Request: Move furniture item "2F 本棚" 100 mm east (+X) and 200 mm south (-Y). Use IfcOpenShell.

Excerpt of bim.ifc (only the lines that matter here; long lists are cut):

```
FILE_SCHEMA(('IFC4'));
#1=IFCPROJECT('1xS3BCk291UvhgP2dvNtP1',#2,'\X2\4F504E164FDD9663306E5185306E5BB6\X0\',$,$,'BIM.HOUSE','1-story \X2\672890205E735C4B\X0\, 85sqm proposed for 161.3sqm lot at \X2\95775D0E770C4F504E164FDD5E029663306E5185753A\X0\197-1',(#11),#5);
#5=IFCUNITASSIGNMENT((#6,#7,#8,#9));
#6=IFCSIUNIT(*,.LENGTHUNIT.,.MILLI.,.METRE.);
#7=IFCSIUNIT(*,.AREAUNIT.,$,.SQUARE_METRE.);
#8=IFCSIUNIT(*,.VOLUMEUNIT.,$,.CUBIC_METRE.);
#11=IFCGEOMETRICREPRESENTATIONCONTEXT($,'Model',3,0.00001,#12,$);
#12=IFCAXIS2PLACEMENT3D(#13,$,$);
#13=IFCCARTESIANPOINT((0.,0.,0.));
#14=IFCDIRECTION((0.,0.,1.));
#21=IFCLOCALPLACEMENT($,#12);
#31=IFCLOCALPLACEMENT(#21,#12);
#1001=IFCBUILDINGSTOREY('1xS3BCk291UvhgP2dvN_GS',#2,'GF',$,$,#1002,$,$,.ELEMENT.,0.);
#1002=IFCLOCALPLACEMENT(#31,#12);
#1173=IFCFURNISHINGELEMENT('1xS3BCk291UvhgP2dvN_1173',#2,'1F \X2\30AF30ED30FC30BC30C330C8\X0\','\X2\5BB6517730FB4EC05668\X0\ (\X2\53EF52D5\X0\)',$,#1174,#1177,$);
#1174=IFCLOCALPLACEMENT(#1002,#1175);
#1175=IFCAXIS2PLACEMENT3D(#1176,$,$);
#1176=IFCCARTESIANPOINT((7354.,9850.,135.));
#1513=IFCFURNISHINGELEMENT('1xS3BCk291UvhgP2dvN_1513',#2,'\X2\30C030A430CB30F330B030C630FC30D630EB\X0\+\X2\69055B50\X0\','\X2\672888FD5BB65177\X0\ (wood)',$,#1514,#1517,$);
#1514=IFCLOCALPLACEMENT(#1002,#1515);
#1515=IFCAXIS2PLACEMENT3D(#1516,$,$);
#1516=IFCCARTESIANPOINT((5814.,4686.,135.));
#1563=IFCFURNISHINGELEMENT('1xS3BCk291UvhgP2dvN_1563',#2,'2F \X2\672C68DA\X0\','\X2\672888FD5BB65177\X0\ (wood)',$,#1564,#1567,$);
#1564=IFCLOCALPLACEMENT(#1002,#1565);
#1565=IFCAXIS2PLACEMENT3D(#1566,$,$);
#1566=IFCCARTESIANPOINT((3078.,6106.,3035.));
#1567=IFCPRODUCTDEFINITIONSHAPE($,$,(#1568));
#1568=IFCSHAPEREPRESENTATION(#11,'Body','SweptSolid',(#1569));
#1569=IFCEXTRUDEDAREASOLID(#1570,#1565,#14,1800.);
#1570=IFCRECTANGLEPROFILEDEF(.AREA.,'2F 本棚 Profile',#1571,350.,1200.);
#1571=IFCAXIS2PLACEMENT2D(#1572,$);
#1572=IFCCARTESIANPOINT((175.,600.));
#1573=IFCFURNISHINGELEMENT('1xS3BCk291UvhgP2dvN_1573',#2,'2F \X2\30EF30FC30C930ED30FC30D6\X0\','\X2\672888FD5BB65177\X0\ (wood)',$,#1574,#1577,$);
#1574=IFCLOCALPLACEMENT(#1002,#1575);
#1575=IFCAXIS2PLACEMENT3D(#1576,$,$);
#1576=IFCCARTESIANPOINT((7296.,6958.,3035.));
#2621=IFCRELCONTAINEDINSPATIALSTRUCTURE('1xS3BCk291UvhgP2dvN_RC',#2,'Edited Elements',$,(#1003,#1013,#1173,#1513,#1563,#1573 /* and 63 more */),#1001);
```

```python
import ifcopenshell
import ifcopenshell.api.geometry
import ifcopenshell.util.placement
import ifcopenshell.util.unit

model = ifcopenshell.open("bim.ifc")
unit_scale = ifcopenshell.util.unit.calculate_unit_scale(model)

item = model.by_id(1563)
matrix = ifcopenshell.util.placement.get_local_placement(item.ObjectPlacement)
matrix[0, 3] += 0.1 / unit_scale
matrix[1, 3] -= 0.2 / unit_scale
ifcopenshell.api.geometry.edit_object_placement(model, product=item, matrix=matrix, is_si=False)

print(ifcopenshell.util.placement.get_local_placement(item.ObjectPlacement).round(3) + 0.0)

model.write("bim_edited.ifc")
```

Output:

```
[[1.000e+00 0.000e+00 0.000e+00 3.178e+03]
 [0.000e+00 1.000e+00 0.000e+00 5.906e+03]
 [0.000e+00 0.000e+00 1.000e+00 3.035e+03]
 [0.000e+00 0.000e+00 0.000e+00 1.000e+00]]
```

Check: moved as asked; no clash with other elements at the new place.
